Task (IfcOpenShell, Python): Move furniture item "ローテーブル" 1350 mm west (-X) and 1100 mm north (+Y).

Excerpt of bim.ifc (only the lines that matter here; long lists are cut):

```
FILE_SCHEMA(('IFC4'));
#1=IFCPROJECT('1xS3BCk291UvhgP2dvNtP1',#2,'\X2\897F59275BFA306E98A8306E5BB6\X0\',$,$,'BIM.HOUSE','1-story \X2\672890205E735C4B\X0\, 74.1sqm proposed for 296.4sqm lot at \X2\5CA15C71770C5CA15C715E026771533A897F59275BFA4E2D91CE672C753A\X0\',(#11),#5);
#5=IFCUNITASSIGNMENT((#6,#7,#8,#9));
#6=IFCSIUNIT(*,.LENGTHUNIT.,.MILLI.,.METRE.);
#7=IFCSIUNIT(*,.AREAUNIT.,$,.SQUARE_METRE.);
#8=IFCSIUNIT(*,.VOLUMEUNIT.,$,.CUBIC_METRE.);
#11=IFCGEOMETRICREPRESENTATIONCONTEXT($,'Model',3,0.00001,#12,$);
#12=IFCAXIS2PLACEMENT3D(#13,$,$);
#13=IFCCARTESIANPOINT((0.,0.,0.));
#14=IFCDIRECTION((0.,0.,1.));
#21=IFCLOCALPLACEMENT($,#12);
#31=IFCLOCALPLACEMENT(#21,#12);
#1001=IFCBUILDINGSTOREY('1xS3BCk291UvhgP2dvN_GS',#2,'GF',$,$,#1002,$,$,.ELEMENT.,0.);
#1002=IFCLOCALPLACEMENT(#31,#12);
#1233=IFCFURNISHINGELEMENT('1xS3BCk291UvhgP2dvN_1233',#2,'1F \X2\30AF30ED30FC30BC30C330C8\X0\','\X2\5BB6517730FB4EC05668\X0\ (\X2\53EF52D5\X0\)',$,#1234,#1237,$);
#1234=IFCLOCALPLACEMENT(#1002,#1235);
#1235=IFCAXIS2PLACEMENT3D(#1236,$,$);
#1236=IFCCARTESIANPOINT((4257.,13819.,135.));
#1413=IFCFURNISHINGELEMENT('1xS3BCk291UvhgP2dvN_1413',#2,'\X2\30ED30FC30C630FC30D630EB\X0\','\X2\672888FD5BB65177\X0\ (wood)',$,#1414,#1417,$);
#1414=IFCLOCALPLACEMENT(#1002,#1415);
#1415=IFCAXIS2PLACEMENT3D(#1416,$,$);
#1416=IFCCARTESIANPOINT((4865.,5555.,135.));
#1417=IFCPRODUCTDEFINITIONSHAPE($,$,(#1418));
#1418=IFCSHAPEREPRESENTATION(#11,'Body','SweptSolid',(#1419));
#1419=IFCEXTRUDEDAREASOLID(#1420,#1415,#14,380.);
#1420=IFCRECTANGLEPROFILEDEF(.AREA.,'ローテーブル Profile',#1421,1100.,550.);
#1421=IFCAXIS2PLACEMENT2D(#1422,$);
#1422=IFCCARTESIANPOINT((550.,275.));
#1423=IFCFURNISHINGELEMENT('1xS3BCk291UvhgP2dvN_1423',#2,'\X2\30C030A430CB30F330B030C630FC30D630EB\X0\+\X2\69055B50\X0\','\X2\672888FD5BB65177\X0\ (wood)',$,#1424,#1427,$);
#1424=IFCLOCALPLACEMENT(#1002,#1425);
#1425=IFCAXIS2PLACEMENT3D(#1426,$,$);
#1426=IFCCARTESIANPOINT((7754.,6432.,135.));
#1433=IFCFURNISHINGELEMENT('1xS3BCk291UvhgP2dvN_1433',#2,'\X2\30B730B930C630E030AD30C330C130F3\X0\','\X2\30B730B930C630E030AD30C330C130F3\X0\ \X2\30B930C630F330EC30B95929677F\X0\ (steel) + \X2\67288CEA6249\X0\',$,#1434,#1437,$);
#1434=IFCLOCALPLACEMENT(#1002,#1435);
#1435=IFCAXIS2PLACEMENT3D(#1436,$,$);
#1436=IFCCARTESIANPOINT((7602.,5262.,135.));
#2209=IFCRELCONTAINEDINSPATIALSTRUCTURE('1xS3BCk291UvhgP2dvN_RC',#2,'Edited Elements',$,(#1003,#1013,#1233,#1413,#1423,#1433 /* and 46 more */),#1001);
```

```python
import ifcopenshell
import ifcopenshell.api.geometry
import ifcopenshell.util.placement
import ifcopenshell.util.unit

model = ifcopenshell.open("bim.ifc")
unit_scale = ifcopenshell.util.unit.calculate_unit_scale(model)

item = model.by_id(1413)
matrix = ifcopenshell.util.placement.get_local_placement(item.ObjectPlacement)
matrix[0, 3] -= 1.35 / unit_scale
matrix[1, 3] += 1.1 / unit_scale
ifcopenshell.api.geometry.edit_object_placement(model, product=item, matrix=matrix, is_si=False)

print(ifcopenshell.util.placement.get_local_placement(item.ObjectPlacement).round(3) + 0.0)

model.write("bim_edited.ifc")
```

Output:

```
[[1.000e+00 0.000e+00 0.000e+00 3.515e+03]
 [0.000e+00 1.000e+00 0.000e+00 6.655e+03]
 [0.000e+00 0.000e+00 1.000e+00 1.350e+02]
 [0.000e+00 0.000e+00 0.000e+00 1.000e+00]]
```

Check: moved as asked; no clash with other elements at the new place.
